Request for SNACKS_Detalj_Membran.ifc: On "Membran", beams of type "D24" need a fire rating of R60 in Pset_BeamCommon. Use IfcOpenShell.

First a look at what the model holds.

```python
import ifcopenshell
import ifcopenshell.util.element

model = ifcopenshell.open("SNACKS_Detalj_Membran.ifc")
print(model.schema)
storey = next(s for s in model.by_type("IfcBuildingStorey") if s.Name == "Membran")
beams = [e for e in ifcopenshell.util.element.get_decomposition(storey) if e.is_a("IfcBeam")]
seen = {}
for e in beams:
    element_type = ifcopenshell.util.element.get_type(e)
    key = (element_type.Name if element_type != e and element_type else None, ifcopenshell.util.element.get_pset(e, "Pset_BeamCommon", "FireRating"))
    seen[key] = seen.get(key, 0) + 1
for (name, value), count in sorted(seen.items(), key=str):
    print(count, "x", name, "|", value)
```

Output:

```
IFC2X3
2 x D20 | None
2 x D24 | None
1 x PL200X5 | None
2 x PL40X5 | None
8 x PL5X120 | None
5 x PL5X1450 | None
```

```python
import ifcopenshell
import ifcopenshell.api.pset
import ifcopenshell.util.element

model = ifcopenshell.open("SNACKS_Detalj_Membran.ifc")

storey = next(s for s in model.by_type("IfcBuildingStorey") if s.Name == "Membran")
beams = [e for e in ifcopenshell.util.element.get_decomposition(storey) if e.is_a("IfcBeam")]

count = 0
for e in beams:
    element_type = ifcopenshell.util.element.get_type(e)
    if element_type in (None, e) or element_type.Name != "D24":
        continue
    # add_pset returns the element's existing set when there is one.
    pset = ifcopenshell.api.pset.add_pset(model, product=e, name="Pset_BeamCommon")
    ifcopenshell.api.pset.edit_pset(model, pset=pset, properties={"FireRating": "R60"})
    count += 1

print(count, "beams updated")

model.write("SNACKS_Detalj_Membran_v2.ifc")
```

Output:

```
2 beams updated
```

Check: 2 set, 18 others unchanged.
